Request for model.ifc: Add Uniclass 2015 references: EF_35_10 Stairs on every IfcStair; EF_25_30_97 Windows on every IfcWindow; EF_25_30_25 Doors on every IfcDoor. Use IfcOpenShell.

First a look at what the model holds.

```python
import ifcopenshell

model = ifcopenshell.open("model.ifc")
print(model.schema)
print("classifications:", [c.Name for c in model.by_type("IfcClassification")])
for ifc_class in ("IfcDoor", "IfcRoof", "IfcStair", "IfcWall", "IfcWindow"):
    print(ifc_class, len(model.by_type(ifc_class)))
```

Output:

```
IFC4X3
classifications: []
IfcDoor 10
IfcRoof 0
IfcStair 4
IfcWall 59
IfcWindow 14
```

```python
import ifcopenshell
import ifcopenshell.api.classification

model = ifcopenshell.open("model.ifc")

system = ifcopenshell.api.classification.add_classification(model, classification="Uniclass 2015")

codes = {
    "IfcStair": ("EF_35_10", "Stairs"),
    "IfcWindow": ("EF_25_30_97", "Windows"),
    "IfcDoor": ("EF_25_30_25", "Doors"),
}
for ifc_class, (code, name) in codes.items():
    products = model.by_type(ifc_class)
    ifcopenshell.api.classification.add_reference(
        model, products=products, classification=system, identification=code, name=name
    )
    print(code, len(products))

model.write("model_v2.ifc")
```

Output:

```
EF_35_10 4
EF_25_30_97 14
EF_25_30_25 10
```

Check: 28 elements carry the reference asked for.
